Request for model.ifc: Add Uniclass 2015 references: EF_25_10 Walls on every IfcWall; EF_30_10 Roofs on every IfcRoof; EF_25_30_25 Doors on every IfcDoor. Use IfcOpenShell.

First a look at what the model holds.

```python
import ifcopenshell

model = ifcopenshell.open("model.ifc")
print(model.schema)
print("classifications:", [c.Name for c in model.by_type("IfcClassification")])
for ifc_class in ("IfcDoor", "IfcRoof", "IfcStair", "IfcWall", "IfcWindow"):
    print(ifc_class, len(model.by_type(ifc_class)))
```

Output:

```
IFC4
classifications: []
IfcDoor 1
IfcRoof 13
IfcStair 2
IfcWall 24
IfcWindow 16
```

```python
import ifcopenshell
import ifcopenshell.api.classification

model = ifcopenshell.open("model.ifc")

system = ifcopenshell.api.classification.add_classification(model, classification="Uniclass 2015")

codes = {
    "IfcWall": ("EF_25_10", "Walls"),
    "IfcRoof": ("EF_30_10", "Roofs"),
    "IfcDoor": ("EF_25_30_25", "Doors"),
}
for ifc_class, (code, name) in codes.items():
    products = model.by_type(ifc_class)
    ifcopenshell.api.classification.add_reference(
        model, products=products, classification=system, identification=code, name=name
    )
    print(code, len(products))

model.write("model-out.ifc")
```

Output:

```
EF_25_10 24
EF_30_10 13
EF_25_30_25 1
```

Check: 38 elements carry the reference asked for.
